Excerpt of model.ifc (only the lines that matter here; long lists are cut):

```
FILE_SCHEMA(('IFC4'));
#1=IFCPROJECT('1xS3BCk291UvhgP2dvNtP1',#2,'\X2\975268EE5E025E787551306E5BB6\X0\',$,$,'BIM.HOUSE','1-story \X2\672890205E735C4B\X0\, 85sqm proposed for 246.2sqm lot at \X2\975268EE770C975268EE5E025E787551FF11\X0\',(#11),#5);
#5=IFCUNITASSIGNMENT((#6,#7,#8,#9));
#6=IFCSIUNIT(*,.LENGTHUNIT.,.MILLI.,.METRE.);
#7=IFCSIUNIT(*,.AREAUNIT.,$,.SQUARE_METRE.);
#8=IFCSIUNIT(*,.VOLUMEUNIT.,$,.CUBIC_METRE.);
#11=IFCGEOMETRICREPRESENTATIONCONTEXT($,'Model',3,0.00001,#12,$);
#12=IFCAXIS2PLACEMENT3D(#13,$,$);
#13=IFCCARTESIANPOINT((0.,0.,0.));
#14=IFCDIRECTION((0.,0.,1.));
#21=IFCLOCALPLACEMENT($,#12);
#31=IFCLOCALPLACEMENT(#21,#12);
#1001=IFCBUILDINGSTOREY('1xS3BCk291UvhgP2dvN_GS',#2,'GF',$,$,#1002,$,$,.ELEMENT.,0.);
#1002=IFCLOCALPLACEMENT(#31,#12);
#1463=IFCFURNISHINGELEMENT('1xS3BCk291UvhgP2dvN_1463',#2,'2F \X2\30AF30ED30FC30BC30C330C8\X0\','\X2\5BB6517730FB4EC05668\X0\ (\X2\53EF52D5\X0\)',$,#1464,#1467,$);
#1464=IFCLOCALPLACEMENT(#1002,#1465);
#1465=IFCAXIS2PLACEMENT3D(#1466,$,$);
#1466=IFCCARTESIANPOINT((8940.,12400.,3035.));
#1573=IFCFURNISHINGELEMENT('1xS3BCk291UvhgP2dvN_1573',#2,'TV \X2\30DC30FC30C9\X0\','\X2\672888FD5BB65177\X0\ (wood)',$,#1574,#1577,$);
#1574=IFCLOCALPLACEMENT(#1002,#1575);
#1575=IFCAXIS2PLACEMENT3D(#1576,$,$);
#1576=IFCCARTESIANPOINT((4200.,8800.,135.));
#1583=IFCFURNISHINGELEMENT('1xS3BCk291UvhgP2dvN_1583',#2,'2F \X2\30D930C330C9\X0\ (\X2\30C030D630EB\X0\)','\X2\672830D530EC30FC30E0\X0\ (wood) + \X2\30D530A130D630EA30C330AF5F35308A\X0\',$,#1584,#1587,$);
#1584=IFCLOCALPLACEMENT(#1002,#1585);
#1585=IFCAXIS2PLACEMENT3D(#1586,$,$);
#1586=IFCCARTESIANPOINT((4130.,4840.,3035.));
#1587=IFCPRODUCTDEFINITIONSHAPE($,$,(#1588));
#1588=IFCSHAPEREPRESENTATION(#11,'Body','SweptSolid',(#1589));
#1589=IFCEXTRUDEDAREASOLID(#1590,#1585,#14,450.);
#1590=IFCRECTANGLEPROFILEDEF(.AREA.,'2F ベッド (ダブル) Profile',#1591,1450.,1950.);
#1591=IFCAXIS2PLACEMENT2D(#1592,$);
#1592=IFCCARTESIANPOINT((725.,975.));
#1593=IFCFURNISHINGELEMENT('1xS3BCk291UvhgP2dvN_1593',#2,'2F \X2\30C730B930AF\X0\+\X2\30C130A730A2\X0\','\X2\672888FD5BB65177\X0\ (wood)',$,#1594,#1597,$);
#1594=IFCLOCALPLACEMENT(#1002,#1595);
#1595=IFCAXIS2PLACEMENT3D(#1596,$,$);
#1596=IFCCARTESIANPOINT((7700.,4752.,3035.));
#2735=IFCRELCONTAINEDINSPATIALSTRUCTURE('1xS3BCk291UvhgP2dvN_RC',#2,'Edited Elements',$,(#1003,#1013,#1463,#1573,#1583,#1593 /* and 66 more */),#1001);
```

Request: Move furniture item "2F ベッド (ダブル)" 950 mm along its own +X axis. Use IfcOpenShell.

```python
import ifcopenshell
import ifcopenshell.api.geometry
import ifcopenshell.util.placement
import ifcopenshell.util.unit

model = ifcopenshell.open("model.ifc")
unit_scale = ifcopenshell.util.unit.calculate_unit_scale(model)

item = model.by_guid("1xS3BCk291UvhgP2dvN_1583")
matrix = ifcopenshell.util.placement.get_local_placement(item.ObjectPlacement)
matrix[:3, 3] += matrix[:3, 0] * 0.95 / unit_scale
ifcopenshell.api.geometry.edit_object_placement(model, product=item, matrix=matrix, is_si=False)

print(ifcopenshell.util.placement.get_local_placement(item.ObjectPlacement).round(3) + 0.0)

model.write("model-out.ifc")
```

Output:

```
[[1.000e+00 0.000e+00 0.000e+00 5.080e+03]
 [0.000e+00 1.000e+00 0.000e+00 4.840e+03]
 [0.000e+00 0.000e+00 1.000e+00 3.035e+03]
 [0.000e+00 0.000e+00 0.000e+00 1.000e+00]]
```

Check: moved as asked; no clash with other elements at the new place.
